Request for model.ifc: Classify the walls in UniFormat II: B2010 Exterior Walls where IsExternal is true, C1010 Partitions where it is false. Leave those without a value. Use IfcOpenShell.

First a look at what the model holds.

```python
import ifcopenshell
import ifcopenshell.util.element

model = ifcopenshell.open("model.ifc")
print(model.schema)
print("classifications:", [c.Name for c in model.by_type("IfcClassification")])
values = [ifcopenshell.util.element.get_pset(e, "Pset_WallCommon", "IsExternal") for e in model.by_type("IfcWall")]
for value in (True, False, None):
    print("IsExternal", value, values.count(value))
```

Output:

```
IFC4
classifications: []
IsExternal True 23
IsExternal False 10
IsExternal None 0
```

```python
import ifcopenshell
import ifcopenshell.api.classification
import ifcopenshell.util.element

model = ifcopenshell.open("model.ifc")

system = ifcopenshell.api.classification.add_classification(model, classification="UniFormat II")

walls = model.by_type("IfcWall")
external = {e: ifcopenshell.util.element.get_pset(e, "Pset_WallCommon", "IsExternal") for e in walls}
for flag, code, name in ((True, "B2010", "Exterior Walls"), (False, "C1010", "Partitions")):
    products = [e for e in walls if external[e] is flag]
    ifcopenshell.api.classification.add_reference(
        model, products=products, classification=system, identification=code, name=name
    )
    print(code, len(products))

model.write("model_edited.ifc")
```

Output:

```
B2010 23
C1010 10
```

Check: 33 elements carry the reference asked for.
